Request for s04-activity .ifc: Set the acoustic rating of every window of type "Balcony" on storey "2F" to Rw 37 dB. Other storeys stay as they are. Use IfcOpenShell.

First a look at what the model holds.

```python
import ifcopenshell
import ifcopenshell.util.element

model = ifcopenshell.open("s04-activity .ifc")
print(model.schema)
storey = next(s for s in model.by_type("IfcBuildingStorey") if s.Name == "2F")
windows = [e for e in ifcopenshell.util.element.get_decomposition(storey) if e.is_a("IfcWindow")]
seen = {}
for e in windows:
    element_type = ifcopenshell.util.element.get_type(e)
    key = (element_type.Name if element_type != e and element_type else None, ifcopenshell.util.element.get_pset(e, "Pset_WindowCommon", "AcousticRating"))
    seen[key] = seen.get(key, 0) + 1
for (name, value), count in sorted(seen.items(), key=str):
    print(count, "x", name, "|", value)
```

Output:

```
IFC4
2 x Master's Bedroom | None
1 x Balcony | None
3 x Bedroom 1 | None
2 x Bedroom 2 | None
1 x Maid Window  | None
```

```python
import ifcopenshell
import ifcopenshell.api.pset
import ifcopenshell.util.element

model = ifcopenshell.open("s04-activity .ifc")

storey = next(s for s in model.by_type("IfcBuildingStorey") if s.Name == "2F")
windows = [e for e in ifcopenshell.util.element.get_decomposition(storey) if e.is_a("IfcWindow")]

count = 0
for e in windows:
    element_type = ifcopenshell.util.element.get_type(e)
    if element_type in (None, e) or element_type.Name != "Balcony":
        continue
    # add_pset returns the element's existing set when there is one.
    pset = ifcopenshell.api.pset.add_pset(model, product=e, name="Pset_WindowCommon")
    ifcopenshell.api.pset.edit_pset(model, pset=pset, properties={"AcousticRating": "Rw 37 dB"})
    count += 1

print(count, "windows updated")

model.write("s04-activity _v2.ifc")
```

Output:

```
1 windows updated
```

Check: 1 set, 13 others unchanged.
